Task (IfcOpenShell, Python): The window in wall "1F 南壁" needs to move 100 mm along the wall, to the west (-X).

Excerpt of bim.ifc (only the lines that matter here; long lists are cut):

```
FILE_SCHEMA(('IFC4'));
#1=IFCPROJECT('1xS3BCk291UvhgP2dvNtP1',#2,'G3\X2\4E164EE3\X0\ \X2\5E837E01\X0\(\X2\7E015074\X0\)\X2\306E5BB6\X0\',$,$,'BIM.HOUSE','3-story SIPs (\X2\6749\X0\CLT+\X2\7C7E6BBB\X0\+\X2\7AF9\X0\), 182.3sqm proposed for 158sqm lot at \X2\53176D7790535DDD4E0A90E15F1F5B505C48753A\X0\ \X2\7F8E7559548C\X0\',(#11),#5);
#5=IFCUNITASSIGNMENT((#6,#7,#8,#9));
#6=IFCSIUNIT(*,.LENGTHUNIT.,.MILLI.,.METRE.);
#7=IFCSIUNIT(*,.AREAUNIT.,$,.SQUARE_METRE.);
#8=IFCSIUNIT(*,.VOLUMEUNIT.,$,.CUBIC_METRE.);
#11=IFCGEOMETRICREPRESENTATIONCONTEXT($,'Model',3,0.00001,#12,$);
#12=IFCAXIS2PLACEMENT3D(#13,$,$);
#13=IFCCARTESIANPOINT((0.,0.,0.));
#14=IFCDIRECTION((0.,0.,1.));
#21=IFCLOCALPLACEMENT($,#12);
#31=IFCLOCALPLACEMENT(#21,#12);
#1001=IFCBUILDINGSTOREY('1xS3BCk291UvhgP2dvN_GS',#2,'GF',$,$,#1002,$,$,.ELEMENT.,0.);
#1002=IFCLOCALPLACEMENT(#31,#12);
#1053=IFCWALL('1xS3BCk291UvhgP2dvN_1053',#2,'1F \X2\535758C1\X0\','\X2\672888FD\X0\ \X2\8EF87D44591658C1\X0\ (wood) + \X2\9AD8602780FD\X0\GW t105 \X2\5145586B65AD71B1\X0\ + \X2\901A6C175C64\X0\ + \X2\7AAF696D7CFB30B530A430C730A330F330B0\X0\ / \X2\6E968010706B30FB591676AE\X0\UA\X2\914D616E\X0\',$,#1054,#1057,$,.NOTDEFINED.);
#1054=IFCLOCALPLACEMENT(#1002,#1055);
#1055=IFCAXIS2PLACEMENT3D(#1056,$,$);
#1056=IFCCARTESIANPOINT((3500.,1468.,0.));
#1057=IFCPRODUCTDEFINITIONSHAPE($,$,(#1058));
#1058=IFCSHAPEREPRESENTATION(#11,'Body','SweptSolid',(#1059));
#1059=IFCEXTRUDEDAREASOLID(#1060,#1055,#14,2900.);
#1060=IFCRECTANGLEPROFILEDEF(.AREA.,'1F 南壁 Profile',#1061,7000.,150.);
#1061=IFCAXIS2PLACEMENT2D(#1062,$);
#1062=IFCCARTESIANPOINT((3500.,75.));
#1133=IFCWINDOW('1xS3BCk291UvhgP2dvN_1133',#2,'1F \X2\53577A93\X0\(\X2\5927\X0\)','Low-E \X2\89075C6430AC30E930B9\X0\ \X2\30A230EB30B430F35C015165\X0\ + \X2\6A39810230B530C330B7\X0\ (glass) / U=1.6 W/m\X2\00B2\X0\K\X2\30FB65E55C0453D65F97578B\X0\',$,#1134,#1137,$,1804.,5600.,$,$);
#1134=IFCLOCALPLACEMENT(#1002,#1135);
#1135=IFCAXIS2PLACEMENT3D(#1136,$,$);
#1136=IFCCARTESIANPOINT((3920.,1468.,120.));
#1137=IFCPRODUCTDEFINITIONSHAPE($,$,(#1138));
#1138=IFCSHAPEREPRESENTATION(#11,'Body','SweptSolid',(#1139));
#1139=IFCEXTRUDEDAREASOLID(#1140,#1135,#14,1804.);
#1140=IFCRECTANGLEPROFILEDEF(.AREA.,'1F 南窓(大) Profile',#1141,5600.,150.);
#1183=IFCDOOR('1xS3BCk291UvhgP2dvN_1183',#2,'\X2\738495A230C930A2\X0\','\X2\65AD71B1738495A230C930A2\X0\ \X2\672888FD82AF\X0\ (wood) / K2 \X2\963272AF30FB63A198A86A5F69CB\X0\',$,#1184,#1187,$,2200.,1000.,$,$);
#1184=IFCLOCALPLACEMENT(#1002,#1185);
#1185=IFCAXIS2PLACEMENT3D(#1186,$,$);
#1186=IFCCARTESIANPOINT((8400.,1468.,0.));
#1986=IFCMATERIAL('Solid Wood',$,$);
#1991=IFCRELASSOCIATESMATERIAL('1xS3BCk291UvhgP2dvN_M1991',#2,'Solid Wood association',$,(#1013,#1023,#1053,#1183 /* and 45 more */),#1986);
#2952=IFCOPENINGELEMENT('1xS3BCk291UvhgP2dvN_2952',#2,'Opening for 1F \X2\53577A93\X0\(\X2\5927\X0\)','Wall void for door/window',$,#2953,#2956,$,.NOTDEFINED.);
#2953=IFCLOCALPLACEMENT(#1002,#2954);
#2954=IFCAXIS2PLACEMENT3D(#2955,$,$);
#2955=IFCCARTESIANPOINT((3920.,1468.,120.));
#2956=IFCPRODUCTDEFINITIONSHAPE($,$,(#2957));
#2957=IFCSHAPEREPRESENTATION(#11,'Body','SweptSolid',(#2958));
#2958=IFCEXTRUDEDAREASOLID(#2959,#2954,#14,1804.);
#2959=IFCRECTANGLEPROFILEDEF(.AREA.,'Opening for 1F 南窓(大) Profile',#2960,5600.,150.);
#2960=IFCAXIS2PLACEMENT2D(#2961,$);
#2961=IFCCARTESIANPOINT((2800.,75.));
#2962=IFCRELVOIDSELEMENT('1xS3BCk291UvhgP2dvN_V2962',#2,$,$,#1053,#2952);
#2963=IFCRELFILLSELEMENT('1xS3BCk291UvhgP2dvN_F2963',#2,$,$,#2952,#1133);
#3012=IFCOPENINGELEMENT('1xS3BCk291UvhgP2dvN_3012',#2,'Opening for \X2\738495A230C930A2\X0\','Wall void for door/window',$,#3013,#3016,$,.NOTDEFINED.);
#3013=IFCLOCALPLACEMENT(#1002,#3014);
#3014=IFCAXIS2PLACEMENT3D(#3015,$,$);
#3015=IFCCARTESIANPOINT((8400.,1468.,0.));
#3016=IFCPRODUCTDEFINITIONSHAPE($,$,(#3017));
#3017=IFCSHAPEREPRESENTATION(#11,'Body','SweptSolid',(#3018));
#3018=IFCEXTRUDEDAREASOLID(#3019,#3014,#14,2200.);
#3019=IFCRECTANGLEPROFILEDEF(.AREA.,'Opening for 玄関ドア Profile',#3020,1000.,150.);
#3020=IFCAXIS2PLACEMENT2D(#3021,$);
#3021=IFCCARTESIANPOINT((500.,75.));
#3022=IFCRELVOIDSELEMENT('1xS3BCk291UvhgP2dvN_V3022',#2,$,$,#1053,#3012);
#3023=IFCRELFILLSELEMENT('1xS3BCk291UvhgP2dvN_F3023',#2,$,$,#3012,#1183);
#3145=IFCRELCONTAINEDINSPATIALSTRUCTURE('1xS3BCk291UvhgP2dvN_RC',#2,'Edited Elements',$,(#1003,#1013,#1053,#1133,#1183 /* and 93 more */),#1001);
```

```python
import ifcopenshell
import ifcopenshell.api.geometry
import ifcopenshell.util.placement

model = ifcopenshell.open("bim.ifc")

window = model.by_guid("1xS3BCk291UvhgP2dvN_1133")
opening = window.FillsVoids[0].RelatingOpeningElement
wall = opening.VoidsElements[0].RelatingBuildingElement

wall_matrix = ifcopenshell.util.placement.get_local_placement(wall.ObjectPlacement)
shift = wall_matrix[:3, 0] * -100.0
before = ifcopenshell.util.placement.get_local_placement(window.ObjectPlacement)[:3, 3].copy()

# The window is not placed relative to its opening, so move both.
for product in (opening, window):
    matrix = ifcopenshell.util.placement.get_local_placement(product.ObjectPlacement)
    matrix[:3, 3] += shift
    ifcopenshell.api.geometry.edit_object_placement(model, product=product, matrix=matrix, is_si=False)

after = ifcopenshell.util.placement.get_local_placement(window.ObjectPlacement)[:3, 3]
print("window moved by", (after - before).round(3) + 0.0)

model.write("bim_rev.ifc")
```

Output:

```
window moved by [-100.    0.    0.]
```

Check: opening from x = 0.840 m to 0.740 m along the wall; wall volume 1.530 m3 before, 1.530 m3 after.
